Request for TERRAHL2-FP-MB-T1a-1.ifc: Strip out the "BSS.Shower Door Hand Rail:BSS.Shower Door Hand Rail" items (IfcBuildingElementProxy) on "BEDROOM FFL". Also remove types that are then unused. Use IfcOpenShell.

First a look at what the model holds.

```python
import ifcopenshell
import ifcopenshell.util.element

model = ifcopenshell.open("TERRAHL2-FP-MB-T1a-1.ifc")
print(model.schema)
storey = next(s for s in model.by_type("IfcBuildingStorey") if s.Name == "BEDROOM FFL")
proxies = [e for e in ifcopenshell.util.element.get_decomposition(storey) if e.is_a("IfcBuildingElementProxy")]
seen = {}
for e in proxies:
    element_type = ifcopenshell.util.element.get_type(e)
    name = element_type.Name if element_type not in (None, e) else None
    seen[name] = seen.get(name, 0) + 1
for name, count in sorted(seen.items(), key=str):
    print(count, "x", name)
```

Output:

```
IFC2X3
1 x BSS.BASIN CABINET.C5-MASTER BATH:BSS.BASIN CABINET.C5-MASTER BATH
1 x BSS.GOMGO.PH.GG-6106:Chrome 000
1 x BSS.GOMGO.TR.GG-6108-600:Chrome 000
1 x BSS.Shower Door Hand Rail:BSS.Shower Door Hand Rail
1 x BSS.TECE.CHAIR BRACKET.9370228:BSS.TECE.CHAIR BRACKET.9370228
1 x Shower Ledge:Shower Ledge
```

```python
import ifcopenshell
import ifcopenshell.api.root
import ifcopenshell.util.element

model = ifcopenshell.open("TERRAHL2-FP-MB-T1a-1.ifc")

storey = next(s for s in model.by_type("IfcBuildingStorey") if s.Name == "BEDROOM FFL")
proxies = [e for e in ifcopenshell.util.element.get_decomposition(storey) if e.is_a("IfcBuildingElementProxy")]
targets = [e for e in proxies if (t := ifcopenshell.util.element.get_type(e)) not in (None, e) and t.Name == "BSS.Shower Door Hand Rail:BSS.Shower Door Hand Rail"]
types = {ifcopenshell.util.element.get_type(e) for e in targets} - {None, *targets}

for e in targets:
    ifcopenshell.api.root.remove_product(model, product=e)
print(len(targets), "removed")

unused = [t for t in types if not ifcopenshell.util.element.get_types(t)]
for t in unused:
    ifcopenshell.api.root.remove_product(model, product=t)
print(len(unused), "unused types removed")

model.write("TERRAHL2-FP-MB-T1a-1_v2.ifc")
```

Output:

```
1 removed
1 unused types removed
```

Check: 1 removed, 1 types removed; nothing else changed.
